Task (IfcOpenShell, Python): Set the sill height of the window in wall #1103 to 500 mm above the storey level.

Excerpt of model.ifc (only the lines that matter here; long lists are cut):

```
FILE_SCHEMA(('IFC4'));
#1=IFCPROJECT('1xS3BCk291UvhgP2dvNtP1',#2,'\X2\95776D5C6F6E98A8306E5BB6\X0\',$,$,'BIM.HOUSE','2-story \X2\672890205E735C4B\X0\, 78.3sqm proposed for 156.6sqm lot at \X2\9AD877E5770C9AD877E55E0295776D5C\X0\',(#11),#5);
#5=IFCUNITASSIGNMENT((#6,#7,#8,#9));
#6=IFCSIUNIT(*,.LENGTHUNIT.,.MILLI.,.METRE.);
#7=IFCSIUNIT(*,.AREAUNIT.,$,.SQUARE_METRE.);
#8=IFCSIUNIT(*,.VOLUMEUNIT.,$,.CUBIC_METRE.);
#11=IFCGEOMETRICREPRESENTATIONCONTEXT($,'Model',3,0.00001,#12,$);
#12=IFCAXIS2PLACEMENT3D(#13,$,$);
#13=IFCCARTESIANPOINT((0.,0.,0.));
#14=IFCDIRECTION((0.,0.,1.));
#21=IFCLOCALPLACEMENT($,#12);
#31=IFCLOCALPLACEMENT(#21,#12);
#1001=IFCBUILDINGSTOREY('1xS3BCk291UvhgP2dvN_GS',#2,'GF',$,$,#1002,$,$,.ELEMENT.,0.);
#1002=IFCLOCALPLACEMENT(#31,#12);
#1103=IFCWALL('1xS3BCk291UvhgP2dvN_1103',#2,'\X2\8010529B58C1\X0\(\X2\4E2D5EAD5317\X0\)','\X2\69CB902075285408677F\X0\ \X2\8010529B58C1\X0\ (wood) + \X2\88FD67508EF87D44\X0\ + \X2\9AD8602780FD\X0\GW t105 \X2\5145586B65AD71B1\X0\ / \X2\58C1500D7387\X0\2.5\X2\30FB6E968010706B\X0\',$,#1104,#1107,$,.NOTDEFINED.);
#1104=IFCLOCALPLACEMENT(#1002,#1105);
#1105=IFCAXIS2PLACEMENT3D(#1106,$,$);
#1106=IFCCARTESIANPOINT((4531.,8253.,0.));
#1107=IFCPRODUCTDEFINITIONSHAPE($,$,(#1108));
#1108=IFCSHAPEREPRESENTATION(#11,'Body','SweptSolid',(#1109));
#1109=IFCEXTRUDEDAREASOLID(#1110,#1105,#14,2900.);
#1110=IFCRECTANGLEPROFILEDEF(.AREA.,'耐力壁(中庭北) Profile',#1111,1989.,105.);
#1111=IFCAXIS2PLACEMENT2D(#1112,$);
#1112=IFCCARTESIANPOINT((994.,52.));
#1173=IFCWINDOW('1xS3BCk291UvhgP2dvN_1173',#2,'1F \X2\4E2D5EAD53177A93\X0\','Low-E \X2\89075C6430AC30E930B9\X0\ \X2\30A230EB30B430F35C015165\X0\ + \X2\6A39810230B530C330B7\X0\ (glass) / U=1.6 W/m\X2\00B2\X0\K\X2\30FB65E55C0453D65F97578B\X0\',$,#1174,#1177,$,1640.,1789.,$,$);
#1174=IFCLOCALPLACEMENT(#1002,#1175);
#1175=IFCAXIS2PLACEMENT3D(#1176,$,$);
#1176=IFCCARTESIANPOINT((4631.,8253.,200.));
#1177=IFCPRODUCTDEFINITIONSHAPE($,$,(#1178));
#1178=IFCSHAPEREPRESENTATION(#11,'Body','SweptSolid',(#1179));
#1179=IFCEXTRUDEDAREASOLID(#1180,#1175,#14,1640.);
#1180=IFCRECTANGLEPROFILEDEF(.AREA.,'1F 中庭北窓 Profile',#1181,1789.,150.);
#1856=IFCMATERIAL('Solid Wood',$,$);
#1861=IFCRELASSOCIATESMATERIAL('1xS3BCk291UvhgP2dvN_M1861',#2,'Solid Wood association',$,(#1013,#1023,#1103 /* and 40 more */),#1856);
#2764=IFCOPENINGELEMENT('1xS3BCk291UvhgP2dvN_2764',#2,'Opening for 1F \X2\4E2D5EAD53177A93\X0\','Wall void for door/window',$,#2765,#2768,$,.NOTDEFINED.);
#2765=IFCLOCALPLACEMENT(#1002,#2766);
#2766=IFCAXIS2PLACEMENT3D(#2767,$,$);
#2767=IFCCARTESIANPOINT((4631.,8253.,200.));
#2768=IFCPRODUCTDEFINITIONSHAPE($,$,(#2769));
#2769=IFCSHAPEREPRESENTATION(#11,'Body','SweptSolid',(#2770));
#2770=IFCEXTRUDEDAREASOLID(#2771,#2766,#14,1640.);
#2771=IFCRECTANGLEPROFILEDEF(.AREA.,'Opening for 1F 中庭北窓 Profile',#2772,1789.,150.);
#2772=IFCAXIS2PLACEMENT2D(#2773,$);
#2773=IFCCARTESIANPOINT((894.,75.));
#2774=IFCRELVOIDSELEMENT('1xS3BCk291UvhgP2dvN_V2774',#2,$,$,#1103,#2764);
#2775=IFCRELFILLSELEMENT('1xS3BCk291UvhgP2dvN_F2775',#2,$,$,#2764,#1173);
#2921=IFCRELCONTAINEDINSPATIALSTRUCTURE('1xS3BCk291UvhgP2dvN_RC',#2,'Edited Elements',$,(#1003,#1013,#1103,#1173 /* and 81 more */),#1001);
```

```python
import numpy as np
import ifcopenshell
import ifcopenshell.api.geometry
import ifcopenshell.geom
import ifcopenshell.util.element
import ifcopenshell.util.placement
import ifcopenshell.util.shape
import ifcopenshell.util.unit

model = ifcopenshell.open("model.ifc")
unit_scale = ifcopenshell.util.unit.calculate_unit_scale(model)

window = model.by_guid("1xS3BCk291UvhgP2dvN_1173")
opening = window.FillsVoids[0].RelatingOpeningElement
storey = ifcopenshell.util.element.get_container(window, ifc_class="IfcBuildingStorey")
level = ifcopenshell.util.placement.get_local_placement(storey.ObjectPlacement)[2, 3]

# The opening's origin need not be at the sill, so measure its lowest point.
shape = ifcopenshell.geom.create_shape(ifcopenshell.geom.settings(), opening)
bottom = ifcopenshell.util.shape.get_shape_bottom_elevation(shape, shape.geometry) / unit_scale
dz = level + 500.0 - bottom

shift = np.array([0.0, 0.0, dz])
# The window is not placed relative to its opening, so move both.
for product in (opening, window):
    matrix = ifcopenshell.util.placement.get_local_placement(product.ObjectPlacement)
    matrix[:3, 3] += shift
    ifcopenshell.api.geometry.edit_object_placement(model, product=product, matrix=matrix, is_si=False)

print(f"moved by {dz * unit_scale:+.3f} m")

model.write("model_updated.ifc")
```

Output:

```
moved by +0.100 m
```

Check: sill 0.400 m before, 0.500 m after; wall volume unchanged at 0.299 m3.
